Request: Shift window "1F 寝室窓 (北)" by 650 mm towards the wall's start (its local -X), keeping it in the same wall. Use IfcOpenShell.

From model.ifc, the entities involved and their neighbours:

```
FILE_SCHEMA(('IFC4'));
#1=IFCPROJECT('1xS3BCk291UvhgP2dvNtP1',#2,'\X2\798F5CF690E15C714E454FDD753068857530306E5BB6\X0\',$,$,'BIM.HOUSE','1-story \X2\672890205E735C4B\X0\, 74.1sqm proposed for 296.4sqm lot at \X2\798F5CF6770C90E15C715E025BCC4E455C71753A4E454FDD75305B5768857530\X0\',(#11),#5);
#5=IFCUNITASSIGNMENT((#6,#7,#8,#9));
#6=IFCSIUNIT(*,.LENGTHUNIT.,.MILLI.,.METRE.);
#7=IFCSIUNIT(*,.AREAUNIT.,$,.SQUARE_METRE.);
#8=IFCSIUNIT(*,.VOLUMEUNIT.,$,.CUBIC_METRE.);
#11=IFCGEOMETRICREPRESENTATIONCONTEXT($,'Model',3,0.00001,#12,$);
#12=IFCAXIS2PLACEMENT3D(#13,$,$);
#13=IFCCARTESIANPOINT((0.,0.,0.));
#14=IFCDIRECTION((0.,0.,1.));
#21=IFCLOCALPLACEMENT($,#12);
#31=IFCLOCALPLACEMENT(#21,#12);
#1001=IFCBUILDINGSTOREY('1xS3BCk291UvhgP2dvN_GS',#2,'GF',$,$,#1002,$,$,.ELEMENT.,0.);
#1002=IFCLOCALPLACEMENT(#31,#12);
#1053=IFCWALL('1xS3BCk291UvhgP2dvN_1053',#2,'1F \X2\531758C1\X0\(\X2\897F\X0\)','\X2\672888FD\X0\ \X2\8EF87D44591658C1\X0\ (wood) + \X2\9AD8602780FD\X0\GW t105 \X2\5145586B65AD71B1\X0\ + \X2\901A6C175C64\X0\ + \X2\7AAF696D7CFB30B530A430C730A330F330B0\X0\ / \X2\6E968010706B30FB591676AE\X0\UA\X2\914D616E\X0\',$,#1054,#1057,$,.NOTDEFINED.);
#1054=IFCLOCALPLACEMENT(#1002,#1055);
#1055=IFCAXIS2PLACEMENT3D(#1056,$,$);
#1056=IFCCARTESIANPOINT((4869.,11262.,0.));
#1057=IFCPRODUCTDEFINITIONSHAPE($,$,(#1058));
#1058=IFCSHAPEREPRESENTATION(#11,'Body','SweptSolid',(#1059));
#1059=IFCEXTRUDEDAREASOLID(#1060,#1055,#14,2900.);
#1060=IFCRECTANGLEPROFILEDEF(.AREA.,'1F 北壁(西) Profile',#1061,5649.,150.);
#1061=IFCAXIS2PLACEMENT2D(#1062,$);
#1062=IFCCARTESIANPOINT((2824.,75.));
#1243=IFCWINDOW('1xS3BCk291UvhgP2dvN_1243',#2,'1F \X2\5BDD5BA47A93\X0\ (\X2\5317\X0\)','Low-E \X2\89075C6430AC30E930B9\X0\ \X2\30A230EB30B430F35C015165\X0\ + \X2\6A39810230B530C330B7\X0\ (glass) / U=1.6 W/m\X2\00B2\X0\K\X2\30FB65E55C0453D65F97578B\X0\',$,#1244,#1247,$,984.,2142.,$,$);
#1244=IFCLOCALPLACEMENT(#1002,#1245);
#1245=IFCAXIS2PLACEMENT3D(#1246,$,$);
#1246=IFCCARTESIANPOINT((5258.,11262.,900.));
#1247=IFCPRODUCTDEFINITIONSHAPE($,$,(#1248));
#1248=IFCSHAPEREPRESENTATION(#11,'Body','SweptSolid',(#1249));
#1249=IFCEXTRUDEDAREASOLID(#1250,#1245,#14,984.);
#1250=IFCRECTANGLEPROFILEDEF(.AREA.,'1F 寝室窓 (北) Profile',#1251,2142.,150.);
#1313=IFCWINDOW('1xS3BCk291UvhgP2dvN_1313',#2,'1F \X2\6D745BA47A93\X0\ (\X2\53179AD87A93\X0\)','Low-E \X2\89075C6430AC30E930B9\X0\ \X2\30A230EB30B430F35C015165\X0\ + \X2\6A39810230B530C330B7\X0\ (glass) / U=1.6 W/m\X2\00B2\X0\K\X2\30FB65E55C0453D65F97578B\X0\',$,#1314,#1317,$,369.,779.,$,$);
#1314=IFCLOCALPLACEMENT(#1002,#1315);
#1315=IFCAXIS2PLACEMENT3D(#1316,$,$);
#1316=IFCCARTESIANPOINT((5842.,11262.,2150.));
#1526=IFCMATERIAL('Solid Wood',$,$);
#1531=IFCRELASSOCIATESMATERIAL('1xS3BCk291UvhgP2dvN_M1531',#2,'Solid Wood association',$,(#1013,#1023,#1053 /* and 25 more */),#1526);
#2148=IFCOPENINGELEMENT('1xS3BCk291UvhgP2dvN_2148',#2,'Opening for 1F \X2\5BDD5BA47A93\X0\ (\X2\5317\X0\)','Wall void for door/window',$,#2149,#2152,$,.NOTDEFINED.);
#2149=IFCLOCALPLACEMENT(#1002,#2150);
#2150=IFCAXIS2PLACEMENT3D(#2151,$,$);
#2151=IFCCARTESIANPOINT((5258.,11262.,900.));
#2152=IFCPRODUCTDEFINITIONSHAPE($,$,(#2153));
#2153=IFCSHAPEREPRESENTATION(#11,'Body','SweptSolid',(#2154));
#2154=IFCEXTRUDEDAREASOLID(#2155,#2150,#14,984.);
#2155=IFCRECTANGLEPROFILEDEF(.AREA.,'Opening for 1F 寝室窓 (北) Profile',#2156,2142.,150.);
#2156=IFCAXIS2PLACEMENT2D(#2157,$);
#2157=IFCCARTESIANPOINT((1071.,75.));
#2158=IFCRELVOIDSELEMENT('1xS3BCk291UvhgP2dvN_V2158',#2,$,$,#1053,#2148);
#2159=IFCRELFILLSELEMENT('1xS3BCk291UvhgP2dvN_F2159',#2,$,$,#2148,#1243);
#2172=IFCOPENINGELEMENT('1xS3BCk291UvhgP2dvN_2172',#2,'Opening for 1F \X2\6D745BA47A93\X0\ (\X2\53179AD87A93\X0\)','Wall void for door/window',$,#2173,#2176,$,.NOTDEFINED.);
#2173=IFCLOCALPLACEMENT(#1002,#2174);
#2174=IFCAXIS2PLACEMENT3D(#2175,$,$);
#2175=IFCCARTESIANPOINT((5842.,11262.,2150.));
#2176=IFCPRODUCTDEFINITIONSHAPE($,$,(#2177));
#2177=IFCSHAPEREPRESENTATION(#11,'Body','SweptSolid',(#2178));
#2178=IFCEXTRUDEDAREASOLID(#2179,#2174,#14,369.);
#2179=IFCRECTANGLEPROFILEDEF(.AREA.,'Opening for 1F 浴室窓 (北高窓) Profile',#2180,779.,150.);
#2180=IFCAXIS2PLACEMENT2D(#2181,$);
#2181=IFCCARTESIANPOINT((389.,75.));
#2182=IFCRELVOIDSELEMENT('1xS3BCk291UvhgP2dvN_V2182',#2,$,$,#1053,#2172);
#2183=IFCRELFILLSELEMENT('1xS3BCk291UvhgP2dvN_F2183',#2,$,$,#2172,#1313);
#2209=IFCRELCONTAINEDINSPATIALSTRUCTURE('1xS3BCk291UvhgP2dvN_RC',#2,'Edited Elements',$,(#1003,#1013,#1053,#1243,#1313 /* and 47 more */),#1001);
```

```python
import ifcopenshell
import ifcopenshell.api.geometry
import ifcopenshell.util.placement

model = ifcopenshell.open("model.ifc")

window = model.by_guid("1xS3BCk291UvhgP2dvN_1243")
opening = window.FillsVoids[0].RelatingOpeningElement
wall = opening.VoidsElements[0].RelatingBuildingElement

wall_matrix = ifcopenshell.util.placement.get_local_placement(wall.ObjectPlacement)
shift = wall_matrix[:3, 0] * -650.0
before = ifcopenshell.util.placement.get_local_placement(window.ObjectPlacement)[:3, 3].copy()

# The window is not placed relative to its opening, so move both.
for product in (opening, window):
    matrix = ifcopenshell.util.placement.get_local_placement(product.ObjectPlacement)
    matrix[:3, 3] += shift
    ifcopenshell.api.geometry.edit_object_placement(model, product=product, matrix=matrix, is_si=False)

after = ifcopenshell.util.placement.get_local_placement(window.ObjectPlacement)[:3, 3]
print("window moved by", (after - before).round(3) + 0.0)

model.write("model_rev.ifc")
```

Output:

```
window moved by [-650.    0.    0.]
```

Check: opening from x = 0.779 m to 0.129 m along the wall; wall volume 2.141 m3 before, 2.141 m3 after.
